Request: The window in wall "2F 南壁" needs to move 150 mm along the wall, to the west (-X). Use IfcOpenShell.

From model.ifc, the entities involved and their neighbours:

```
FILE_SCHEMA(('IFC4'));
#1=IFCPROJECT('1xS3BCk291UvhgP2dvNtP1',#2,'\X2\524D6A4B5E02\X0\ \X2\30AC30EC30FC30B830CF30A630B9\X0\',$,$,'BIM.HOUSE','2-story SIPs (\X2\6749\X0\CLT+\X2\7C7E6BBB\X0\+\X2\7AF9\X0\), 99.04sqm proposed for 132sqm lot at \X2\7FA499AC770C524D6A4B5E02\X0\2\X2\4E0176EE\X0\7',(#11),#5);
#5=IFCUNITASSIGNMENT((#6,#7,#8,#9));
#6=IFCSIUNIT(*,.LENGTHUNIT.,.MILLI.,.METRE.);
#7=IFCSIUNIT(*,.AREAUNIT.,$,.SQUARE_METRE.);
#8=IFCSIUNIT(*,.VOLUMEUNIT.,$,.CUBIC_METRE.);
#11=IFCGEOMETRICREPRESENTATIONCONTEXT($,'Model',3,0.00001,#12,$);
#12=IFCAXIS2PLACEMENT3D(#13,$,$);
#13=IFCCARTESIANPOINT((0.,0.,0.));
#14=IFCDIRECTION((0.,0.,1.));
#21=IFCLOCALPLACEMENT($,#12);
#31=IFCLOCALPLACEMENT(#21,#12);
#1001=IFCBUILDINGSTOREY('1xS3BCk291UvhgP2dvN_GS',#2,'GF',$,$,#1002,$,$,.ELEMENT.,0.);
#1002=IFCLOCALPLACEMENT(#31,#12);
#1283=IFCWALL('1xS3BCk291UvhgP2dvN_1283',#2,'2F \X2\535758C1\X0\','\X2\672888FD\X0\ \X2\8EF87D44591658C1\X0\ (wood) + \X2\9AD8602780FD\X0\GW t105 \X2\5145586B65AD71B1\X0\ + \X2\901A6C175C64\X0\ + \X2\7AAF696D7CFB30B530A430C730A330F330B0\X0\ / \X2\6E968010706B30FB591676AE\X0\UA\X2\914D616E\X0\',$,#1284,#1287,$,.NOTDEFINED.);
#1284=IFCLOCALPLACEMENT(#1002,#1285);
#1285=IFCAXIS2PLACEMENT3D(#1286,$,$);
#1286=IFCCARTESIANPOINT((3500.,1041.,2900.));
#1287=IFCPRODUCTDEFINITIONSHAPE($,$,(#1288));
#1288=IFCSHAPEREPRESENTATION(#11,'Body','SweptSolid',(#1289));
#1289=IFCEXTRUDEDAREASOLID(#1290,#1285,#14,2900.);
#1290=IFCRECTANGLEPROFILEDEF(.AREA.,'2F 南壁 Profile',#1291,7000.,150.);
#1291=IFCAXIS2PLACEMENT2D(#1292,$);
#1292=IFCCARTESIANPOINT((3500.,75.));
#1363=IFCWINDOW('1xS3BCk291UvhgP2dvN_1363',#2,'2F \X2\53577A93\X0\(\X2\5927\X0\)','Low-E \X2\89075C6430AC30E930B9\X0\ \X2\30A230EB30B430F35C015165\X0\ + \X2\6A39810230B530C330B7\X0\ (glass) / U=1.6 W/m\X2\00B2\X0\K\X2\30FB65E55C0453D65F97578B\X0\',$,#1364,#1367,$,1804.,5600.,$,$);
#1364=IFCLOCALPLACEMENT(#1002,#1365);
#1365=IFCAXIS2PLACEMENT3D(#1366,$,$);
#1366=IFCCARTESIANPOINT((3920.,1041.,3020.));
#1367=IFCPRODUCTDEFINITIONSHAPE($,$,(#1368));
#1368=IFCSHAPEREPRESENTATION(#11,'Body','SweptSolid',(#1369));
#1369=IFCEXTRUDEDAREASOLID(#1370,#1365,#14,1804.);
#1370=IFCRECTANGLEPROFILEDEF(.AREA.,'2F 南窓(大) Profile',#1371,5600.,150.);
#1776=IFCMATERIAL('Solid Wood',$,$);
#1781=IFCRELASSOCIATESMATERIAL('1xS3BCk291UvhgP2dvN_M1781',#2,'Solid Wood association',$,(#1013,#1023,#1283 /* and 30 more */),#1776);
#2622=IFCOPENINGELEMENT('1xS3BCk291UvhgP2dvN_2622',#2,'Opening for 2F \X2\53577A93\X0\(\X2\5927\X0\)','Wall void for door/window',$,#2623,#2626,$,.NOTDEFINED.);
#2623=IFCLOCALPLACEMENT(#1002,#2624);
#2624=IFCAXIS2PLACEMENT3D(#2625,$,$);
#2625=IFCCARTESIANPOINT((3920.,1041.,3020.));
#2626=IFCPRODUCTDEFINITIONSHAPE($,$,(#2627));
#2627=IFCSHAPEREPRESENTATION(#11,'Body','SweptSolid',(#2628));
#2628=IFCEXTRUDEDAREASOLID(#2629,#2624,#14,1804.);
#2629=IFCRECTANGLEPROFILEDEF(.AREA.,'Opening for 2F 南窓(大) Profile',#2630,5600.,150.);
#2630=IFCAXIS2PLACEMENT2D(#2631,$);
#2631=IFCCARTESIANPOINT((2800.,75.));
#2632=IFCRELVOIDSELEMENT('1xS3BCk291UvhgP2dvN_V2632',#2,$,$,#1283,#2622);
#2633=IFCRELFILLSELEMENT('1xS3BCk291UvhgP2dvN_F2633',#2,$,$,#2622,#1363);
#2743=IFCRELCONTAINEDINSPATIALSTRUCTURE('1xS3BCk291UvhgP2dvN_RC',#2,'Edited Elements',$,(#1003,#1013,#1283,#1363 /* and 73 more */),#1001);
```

```python
import ifcopenshell
import ifcopenshell.api.geometry
import ifcopenshell.util.placement
import ifcopenshell.util.unit

model = ifcopenshell.open("model.ifc")
unit_scale = ifcopenshell.util.unit.calculate_unit_scale(model)

window = model.by_id(1363)
opening = window.FillsVoids[0].RelatingOpeningElement
wall = opening.VoidsElements[0].RelatingBuildingElement

wall_matrix = ifcopenshell.util.placement.get_local_placement(wall.ObjectPlacement)
shift = wall_matrix[:3, 0] * -0.15 / unit_scale
before = ifcopenshell.util.placement.get_local_placement(window.ObjectPlacement)[:3, 3].copy()

# The window is not placed relative to its opening, so move both.
for product in (opening, window):
    matrix = ifcopenshell.util.placement.get_local_placement(product.ObjectPlacement)
    matrix[:3, 3] += shift
    ifcopenshell.api.geometry.edit_object_placement(model, product=product, matrix=matrix, is_si=False)

after = ifcopenshell.util.placement.get_local_placement(window.ObjectPlacement)[:3, 3]
print("window moved by", (after - before).round(3) + 0.0)

model.write("model_rev.ifc")
```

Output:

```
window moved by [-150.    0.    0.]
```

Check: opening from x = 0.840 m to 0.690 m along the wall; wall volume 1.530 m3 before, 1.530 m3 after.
